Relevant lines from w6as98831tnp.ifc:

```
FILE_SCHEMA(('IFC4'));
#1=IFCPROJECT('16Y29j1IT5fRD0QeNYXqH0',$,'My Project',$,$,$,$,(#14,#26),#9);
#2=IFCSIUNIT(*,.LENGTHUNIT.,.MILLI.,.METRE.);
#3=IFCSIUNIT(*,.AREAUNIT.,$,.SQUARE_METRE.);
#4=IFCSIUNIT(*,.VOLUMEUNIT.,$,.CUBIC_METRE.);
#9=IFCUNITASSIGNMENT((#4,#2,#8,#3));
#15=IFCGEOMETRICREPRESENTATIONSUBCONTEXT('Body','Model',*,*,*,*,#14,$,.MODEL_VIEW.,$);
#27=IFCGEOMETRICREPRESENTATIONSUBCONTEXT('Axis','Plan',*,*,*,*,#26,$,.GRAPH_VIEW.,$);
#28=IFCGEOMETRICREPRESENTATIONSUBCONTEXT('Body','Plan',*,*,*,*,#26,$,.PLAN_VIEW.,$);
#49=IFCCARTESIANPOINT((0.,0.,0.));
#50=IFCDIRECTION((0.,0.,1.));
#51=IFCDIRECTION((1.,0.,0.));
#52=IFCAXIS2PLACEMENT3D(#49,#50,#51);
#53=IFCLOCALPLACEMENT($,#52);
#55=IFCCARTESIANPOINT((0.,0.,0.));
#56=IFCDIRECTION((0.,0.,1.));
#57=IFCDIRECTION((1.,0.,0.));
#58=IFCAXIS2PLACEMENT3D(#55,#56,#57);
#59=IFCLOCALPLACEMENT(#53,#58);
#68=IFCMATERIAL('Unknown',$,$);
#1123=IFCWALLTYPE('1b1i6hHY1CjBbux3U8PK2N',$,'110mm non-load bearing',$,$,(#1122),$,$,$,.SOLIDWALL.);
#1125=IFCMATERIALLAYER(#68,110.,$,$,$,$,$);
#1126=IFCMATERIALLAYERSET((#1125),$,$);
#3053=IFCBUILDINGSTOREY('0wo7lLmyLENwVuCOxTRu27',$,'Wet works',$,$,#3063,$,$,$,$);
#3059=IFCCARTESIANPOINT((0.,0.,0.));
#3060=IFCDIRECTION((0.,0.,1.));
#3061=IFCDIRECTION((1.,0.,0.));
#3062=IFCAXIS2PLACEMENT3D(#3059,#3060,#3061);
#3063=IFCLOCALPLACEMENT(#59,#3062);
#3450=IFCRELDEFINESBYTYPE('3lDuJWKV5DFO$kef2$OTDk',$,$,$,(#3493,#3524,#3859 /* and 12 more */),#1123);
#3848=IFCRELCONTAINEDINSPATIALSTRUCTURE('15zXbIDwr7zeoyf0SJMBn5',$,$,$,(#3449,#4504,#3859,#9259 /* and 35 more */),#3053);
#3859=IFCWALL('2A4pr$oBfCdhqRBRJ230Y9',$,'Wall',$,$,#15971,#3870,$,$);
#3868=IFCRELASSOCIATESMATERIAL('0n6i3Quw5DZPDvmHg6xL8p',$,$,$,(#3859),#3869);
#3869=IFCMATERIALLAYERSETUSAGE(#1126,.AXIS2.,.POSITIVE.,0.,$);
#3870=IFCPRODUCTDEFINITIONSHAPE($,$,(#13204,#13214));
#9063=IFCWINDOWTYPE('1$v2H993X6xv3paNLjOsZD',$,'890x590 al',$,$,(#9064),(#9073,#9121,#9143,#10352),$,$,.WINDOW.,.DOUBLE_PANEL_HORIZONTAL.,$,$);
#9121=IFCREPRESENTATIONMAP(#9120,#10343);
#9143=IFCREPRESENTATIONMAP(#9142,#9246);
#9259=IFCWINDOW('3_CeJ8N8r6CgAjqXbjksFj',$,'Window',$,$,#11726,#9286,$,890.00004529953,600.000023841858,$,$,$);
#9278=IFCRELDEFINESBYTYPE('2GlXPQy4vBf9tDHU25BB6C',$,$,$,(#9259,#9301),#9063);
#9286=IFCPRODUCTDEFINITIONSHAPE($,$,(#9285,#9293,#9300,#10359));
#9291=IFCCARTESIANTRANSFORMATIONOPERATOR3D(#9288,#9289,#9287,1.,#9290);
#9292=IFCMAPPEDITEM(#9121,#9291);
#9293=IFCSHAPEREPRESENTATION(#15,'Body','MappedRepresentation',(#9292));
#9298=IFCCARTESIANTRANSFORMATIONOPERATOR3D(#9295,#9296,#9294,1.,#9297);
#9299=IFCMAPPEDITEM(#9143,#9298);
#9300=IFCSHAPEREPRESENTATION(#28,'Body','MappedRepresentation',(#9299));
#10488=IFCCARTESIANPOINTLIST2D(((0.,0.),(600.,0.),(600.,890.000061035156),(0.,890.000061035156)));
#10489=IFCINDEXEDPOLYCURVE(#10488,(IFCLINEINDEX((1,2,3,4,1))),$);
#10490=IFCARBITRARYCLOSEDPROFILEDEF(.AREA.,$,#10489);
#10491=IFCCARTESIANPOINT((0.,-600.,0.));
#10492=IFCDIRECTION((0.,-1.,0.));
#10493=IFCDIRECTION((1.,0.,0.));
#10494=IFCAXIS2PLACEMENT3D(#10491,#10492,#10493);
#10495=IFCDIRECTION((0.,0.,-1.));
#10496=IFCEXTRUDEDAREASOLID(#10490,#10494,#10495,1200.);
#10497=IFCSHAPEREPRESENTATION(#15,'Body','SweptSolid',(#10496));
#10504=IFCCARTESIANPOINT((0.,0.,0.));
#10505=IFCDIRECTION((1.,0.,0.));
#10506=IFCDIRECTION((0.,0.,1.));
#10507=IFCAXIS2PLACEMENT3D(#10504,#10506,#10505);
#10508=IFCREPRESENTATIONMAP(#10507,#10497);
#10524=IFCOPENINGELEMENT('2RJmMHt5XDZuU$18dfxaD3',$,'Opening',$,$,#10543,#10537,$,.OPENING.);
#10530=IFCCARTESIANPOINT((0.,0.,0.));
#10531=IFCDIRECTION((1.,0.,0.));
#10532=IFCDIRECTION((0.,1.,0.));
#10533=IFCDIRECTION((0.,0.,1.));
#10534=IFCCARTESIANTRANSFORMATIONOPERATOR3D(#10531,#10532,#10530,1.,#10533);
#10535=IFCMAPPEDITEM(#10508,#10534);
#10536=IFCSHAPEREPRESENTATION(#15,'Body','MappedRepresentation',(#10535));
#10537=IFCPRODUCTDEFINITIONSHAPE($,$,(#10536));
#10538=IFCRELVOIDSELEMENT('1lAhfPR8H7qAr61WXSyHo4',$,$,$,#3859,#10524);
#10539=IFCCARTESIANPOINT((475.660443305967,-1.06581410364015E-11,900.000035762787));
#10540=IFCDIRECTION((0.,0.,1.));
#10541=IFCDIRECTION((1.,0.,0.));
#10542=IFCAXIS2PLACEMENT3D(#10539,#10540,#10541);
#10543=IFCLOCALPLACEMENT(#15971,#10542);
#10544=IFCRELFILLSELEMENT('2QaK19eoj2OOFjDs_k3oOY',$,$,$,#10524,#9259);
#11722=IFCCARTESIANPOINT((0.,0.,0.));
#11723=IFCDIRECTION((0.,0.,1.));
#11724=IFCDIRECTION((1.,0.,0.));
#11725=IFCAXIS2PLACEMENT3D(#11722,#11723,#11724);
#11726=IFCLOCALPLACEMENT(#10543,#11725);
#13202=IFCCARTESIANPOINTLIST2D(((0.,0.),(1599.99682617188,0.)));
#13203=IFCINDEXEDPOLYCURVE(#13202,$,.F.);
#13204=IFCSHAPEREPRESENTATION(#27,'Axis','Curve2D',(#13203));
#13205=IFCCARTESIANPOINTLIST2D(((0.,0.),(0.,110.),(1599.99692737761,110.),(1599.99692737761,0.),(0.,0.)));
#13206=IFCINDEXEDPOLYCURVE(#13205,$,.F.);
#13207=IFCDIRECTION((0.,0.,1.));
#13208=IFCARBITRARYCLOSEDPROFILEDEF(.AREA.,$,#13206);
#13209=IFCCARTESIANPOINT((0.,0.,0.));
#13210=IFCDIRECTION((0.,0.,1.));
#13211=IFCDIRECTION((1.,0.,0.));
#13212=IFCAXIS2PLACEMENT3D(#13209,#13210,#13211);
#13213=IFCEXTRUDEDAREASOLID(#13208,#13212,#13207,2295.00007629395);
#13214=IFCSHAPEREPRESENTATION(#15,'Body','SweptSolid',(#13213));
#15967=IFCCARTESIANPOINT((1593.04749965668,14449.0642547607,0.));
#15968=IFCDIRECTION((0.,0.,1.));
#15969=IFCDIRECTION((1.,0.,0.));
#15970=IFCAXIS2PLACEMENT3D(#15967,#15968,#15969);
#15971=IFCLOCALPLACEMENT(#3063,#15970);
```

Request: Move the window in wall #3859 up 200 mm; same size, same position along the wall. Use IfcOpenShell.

```python
import numpy as np
import ifcopenshell
import ifcopenshell.api.geometry
import ifcopenshell.util.placement
import ifcopenshell.util.unit

model = ifcopenshell.open("w6as98831tnp.ifc")
unit_scale = ifcopenshell.util.unit.calculate_unit_scale(model)

window = model.by_guid("3_CeJ8N8r6CgAjqXbjksFj")
opening = window.FillsVoids[0].RelatingOpeningElement
dz = 0.2 / unit_scale

shift = np.array([0.0, 0.0, dz])
# The window is placed relative to its opening, so it follows when the opening moves.
matrix = ifcopenshell.util.placement.get_local_placement(opening.ObjectPlacement)
matrix[:3, 3] += shift
ifcopenshell.api.geometry.edit_object_placement(
    model, product=opening, matrix=matrix, is_si=False, should_transform_children=True
)

print(f"moved by {dz * unit_scale:+.3f} m")

model.write("w6as98831tnp-out.ifc")
```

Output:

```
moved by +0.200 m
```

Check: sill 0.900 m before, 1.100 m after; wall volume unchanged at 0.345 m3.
